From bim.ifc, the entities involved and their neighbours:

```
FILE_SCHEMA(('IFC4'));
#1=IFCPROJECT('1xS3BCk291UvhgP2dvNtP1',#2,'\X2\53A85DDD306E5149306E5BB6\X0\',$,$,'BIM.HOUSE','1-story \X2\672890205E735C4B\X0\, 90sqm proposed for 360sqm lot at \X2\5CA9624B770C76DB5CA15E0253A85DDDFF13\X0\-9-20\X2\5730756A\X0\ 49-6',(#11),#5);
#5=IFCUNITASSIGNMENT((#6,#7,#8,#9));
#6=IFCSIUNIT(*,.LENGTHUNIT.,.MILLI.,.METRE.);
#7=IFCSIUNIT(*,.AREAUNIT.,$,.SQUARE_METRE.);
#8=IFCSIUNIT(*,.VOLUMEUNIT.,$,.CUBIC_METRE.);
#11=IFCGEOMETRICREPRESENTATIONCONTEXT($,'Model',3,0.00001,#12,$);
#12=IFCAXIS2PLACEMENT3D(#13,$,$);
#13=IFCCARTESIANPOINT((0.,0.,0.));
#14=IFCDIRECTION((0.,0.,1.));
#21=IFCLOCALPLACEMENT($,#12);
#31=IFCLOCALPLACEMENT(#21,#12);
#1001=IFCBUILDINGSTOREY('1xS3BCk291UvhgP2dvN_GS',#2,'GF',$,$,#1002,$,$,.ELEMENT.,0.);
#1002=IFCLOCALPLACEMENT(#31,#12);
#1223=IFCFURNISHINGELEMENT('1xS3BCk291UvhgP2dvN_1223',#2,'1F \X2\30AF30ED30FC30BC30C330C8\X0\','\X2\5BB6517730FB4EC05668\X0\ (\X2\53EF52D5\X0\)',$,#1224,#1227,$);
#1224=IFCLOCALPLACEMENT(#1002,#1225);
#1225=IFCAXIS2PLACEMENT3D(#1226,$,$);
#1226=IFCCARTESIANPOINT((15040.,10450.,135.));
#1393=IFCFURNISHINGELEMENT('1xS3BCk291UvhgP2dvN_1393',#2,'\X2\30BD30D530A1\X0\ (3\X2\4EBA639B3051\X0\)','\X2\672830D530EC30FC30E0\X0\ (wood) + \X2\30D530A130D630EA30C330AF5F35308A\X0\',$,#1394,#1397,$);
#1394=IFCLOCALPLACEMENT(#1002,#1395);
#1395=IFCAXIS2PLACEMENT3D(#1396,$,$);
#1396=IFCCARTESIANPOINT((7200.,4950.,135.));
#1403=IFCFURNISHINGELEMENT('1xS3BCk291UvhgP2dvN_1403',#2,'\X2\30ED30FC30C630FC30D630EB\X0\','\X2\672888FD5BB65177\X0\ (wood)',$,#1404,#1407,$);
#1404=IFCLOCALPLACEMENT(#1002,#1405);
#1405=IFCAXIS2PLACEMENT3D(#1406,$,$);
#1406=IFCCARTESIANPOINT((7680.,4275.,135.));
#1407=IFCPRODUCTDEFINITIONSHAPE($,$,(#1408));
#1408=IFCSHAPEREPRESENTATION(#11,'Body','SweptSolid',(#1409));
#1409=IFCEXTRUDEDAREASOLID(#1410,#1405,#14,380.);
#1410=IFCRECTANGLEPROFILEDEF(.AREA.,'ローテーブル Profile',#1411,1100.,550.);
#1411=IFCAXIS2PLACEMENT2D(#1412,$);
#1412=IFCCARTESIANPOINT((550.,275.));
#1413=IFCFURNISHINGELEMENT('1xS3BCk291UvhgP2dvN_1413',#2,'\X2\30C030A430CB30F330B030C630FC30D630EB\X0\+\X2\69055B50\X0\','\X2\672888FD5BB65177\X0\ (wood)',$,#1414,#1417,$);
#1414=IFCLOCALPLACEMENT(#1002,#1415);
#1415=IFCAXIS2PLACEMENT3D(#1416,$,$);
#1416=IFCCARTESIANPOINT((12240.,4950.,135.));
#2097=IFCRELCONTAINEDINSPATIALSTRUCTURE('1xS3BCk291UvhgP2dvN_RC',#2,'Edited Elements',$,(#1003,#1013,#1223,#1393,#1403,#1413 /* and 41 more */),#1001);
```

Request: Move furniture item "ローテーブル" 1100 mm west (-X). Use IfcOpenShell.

```python
import ifcopenshell
import ifcopenshell.api.geometry
import ifcopenshell.util.placement

model = ifcopenshell.open("bim.ifc")

item = model.by_id(1403)
matrix = ifcopenshell.util.placement.get_local_placement(item.ObjectPlacement)
matrix[0, 3] -= 1100.0
ifcopenshell.api.geometry.edit_object_placement(model, product=item, matrix=matrix, is_si=False)

print(ifcopenshell.util.placement.get_local_placement(item.ObjectPlacement).round(3) + 0.0)

model.write("bim-out.ifc")
```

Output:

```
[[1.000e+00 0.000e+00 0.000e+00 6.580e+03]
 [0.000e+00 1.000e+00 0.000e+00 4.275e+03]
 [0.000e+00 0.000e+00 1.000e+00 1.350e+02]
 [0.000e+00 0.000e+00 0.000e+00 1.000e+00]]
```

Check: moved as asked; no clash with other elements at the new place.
